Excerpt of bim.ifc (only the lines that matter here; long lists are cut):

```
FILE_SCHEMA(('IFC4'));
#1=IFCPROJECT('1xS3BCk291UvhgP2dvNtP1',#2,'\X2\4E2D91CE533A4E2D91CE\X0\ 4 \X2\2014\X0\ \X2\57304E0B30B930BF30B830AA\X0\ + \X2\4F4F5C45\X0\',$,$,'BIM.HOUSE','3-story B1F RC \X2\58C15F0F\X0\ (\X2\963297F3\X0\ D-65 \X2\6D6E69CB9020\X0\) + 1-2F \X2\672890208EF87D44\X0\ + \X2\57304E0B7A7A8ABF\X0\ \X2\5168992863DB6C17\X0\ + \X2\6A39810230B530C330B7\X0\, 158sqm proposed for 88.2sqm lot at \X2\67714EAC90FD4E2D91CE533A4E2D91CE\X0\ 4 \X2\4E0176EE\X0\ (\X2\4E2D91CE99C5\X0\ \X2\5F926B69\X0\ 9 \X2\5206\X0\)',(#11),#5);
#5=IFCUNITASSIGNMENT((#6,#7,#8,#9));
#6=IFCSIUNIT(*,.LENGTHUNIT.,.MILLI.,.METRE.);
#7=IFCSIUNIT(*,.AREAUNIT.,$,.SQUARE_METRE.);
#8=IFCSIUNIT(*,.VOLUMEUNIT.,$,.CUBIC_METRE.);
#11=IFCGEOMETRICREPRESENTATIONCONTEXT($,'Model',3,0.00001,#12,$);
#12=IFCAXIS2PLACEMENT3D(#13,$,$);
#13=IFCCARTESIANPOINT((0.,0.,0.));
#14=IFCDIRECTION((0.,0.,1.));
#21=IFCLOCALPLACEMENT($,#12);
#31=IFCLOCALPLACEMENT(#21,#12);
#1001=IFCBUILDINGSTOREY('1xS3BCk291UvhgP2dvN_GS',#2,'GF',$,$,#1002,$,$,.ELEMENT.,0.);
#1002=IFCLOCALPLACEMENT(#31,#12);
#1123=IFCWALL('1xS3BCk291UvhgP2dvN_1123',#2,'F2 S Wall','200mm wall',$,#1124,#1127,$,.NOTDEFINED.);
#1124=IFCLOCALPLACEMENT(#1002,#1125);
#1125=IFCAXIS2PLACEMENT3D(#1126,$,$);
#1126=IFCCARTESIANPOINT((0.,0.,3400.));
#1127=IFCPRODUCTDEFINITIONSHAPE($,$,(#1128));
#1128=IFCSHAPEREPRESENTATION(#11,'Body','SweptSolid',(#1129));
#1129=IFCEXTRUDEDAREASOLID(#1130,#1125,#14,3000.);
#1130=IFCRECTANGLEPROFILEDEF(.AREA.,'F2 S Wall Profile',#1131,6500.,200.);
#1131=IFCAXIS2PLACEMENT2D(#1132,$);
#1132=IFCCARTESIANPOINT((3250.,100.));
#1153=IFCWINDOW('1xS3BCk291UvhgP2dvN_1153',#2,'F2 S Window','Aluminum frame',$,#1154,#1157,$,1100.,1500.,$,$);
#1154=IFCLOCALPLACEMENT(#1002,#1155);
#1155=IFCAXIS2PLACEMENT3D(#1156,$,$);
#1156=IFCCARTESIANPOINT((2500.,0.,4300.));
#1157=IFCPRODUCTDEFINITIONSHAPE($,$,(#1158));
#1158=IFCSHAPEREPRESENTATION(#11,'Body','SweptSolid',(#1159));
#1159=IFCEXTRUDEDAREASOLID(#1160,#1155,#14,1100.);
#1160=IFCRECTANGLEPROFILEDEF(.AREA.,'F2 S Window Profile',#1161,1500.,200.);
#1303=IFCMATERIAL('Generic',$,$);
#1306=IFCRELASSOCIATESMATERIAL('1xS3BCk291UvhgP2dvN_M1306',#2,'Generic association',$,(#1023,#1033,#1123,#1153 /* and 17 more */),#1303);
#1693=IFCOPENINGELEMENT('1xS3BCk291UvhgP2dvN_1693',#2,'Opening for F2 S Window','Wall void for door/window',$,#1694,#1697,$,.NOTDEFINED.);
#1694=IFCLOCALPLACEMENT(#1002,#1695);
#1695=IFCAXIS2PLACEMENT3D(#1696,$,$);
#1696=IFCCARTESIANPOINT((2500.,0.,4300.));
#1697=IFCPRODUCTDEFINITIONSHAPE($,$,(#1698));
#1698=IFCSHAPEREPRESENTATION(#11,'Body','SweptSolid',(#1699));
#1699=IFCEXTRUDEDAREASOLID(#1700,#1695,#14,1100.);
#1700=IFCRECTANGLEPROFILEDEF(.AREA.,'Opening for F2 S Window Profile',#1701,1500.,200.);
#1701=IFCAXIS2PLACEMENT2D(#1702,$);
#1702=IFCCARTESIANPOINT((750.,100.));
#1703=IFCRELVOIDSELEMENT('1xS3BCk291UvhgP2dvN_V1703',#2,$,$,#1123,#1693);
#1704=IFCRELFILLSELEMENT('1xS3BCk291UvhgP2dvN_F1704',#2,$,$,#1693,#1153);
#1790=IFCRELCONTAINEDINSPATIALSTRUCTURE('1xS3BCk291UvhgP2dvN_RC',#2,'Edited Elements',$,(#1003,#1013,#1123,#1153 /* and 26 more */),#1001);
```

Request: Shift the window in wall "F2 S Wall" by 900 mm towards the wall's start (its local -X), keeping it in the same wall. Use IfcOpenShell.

```python
import ifcopenshell
import ifcopenshell.api.geometry
import ifcopenshell.util.placement
import ifcopenshell.util.unit

model = ifcopenshell.open("bim.ifc")
unit_scale = ifcopenshell.util.unit.calculate_unit_scale(model)

window = model.by_guid("1xS3BCk291UvhgP2dvN_1153")
opening = window.FillsVoids[0].RelatingOpeningElement
wall = opening.VoidsElements[0].RelatingBuildingElement

wall_matrix = ifcopenshell.util.placement.get_local_placement(wall.ObjectPlacement)
shift = wall_matrix[:3, 0] * -0.9 / unit_scale
before = ifcopenshell.util.placement.get_local_placement(window.ObjectPlacement)[:3, 3].copy()

# The window is not placed relative to its opening, so move both.
for product in (opening, window):
    matrix = ifcopenshell.util.placement.get_local_placement(product.ObjectPlacement)
    matrix[:3, 3] += shift
    ifcopenshell.api.geometry.edit_object_placement(model, product=product, matrix=matrix, is_si=False)

after = ifcopenshell.util.placement.get_local_placement(window.ObjectPlacement)[:3, 3]
print("window moved by", (after - before).round(3) + 0.0)

model.write("bim_v2.ifc")
```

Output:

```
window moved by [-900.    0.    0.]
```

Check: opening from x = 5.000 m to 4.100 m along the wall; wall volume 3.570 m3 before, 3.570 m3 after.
